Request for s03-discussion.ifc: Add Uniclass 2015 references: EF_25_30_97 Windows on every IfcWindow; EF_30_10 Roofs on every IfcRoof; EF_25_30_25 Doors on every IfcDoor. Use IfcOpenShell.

First a look at what the model holds.

```python
import ifcopenshell

model = ifcopenshell.open("s03-discussion.ifc")
print(model.schema)
print("classifications:", [c.Name for c in model.by_type("IfcClassification")])
for ifc_class in ("IfcDoor", "IfcRoof", "IfcStair", "IfcWall", "IfcWindow"):
    print(ifc_class, len(model.by_type(ifc_class)))
```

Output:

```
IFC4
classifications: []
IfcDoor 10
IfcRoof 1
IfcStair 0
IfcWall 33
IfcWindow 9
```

```python
import ifcopenshell
import ifcopenshell.api.classification

model = ifcopenshell.open("s03-discussion.ifc")

system = ifcopenshell.api.classification.add_classification(model, classification="Uniclass 2015")

codes = {
    "IfcWindow": ("EF_25_30_97", "Windows"),
    "IfcRoof": ("EF_30_10", "Roofs"),
    "IfcDoor": ("EF_25_30_25", "Doors"),
}
for ifc_class, (code, name) in codes.items():
    products = model.by_type(ifc_class)
    ifcopenshell.api.classification.add_reference(
        model, products=products, classification=system, identification=code, name=name
    )
    print(code, len(products))

model.write("s03-discussion_edited.ifc")
```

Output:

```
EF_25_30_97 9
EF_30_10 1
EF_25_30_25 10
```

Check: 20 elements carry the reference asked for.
